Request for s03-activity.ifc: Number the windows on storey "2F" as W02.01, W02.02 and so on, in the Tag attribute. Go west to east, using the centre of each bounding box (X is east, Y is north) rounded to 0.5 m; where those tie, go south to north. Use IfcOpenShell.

First a look at what the model holds.

```python
import ifcopenshell
import ifcopenshell.util.element
import ifcopenshell.util.placement

model = ifcopenshell.open("s03-activity.ifc")
print(model.schema)
storey = next(s for s in model.by_type("IfcBuildingStorey") if s.Name == "2F")
windows = [e for e in ifcopenshell.util.element.get_decomposition(storey) if e.is_a("IfcWindow")]
for e in sorted(windows, key=lambda e: e.id()):
    origin = ifcopenshell.util.placement.get_local_placement(e.ObjectPlacement)[:3, 3]
    print(e.id(), e.Tag, e.Name, origin.round(2) + 0.0, sep=" | ")
```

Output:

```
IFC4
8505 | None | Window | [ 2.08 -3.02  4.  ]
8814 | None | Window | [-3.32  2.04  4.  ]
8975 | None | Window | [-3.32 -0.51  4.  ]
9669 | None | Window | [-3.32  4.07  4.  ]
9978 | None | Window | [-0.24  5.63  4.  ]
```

```python
import ifcopenshell
import ifcopenshell.geom
import ifcopenshell.util.element
import ifcopenshell.util.shape

model = ifcopenshell.open("s03-activity.ifc")
settings = ifcopenshell.geom.settings()
settings.set("use-world-coords", True)


def centre(element):
    shape = ifcopenshell.geom.create_shape(settings, element)
    return ifcopenshell.util.shape.get_bbox_centroid(shape.geometry)


storey = next(s for s in model.by_type("IfcBuildingStorey") if s.Name == "2F")
windows = [e for e in ifcopenshell.util.element.get_decomposition(storey) if e.is_a("IfcWindow")]

# Insertion points can sit at a corner or the storey origin, so sort by the geometry (in metres).
centres = {e: centre(e) for e in windows}
windows.sort(key=lambda e: (round(centres[e][0] / 0.5), centres[e][1]))

for i, e in enumerate(windows, start=1):
    number = f"W02.{i:02d}"
    e.Tag = number
    print(e.id(), number)

model.write("s03-activity_v2.ifc")
```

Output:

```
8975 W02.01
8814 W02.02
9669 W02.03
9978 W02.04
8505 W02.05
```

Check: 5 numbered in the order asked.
